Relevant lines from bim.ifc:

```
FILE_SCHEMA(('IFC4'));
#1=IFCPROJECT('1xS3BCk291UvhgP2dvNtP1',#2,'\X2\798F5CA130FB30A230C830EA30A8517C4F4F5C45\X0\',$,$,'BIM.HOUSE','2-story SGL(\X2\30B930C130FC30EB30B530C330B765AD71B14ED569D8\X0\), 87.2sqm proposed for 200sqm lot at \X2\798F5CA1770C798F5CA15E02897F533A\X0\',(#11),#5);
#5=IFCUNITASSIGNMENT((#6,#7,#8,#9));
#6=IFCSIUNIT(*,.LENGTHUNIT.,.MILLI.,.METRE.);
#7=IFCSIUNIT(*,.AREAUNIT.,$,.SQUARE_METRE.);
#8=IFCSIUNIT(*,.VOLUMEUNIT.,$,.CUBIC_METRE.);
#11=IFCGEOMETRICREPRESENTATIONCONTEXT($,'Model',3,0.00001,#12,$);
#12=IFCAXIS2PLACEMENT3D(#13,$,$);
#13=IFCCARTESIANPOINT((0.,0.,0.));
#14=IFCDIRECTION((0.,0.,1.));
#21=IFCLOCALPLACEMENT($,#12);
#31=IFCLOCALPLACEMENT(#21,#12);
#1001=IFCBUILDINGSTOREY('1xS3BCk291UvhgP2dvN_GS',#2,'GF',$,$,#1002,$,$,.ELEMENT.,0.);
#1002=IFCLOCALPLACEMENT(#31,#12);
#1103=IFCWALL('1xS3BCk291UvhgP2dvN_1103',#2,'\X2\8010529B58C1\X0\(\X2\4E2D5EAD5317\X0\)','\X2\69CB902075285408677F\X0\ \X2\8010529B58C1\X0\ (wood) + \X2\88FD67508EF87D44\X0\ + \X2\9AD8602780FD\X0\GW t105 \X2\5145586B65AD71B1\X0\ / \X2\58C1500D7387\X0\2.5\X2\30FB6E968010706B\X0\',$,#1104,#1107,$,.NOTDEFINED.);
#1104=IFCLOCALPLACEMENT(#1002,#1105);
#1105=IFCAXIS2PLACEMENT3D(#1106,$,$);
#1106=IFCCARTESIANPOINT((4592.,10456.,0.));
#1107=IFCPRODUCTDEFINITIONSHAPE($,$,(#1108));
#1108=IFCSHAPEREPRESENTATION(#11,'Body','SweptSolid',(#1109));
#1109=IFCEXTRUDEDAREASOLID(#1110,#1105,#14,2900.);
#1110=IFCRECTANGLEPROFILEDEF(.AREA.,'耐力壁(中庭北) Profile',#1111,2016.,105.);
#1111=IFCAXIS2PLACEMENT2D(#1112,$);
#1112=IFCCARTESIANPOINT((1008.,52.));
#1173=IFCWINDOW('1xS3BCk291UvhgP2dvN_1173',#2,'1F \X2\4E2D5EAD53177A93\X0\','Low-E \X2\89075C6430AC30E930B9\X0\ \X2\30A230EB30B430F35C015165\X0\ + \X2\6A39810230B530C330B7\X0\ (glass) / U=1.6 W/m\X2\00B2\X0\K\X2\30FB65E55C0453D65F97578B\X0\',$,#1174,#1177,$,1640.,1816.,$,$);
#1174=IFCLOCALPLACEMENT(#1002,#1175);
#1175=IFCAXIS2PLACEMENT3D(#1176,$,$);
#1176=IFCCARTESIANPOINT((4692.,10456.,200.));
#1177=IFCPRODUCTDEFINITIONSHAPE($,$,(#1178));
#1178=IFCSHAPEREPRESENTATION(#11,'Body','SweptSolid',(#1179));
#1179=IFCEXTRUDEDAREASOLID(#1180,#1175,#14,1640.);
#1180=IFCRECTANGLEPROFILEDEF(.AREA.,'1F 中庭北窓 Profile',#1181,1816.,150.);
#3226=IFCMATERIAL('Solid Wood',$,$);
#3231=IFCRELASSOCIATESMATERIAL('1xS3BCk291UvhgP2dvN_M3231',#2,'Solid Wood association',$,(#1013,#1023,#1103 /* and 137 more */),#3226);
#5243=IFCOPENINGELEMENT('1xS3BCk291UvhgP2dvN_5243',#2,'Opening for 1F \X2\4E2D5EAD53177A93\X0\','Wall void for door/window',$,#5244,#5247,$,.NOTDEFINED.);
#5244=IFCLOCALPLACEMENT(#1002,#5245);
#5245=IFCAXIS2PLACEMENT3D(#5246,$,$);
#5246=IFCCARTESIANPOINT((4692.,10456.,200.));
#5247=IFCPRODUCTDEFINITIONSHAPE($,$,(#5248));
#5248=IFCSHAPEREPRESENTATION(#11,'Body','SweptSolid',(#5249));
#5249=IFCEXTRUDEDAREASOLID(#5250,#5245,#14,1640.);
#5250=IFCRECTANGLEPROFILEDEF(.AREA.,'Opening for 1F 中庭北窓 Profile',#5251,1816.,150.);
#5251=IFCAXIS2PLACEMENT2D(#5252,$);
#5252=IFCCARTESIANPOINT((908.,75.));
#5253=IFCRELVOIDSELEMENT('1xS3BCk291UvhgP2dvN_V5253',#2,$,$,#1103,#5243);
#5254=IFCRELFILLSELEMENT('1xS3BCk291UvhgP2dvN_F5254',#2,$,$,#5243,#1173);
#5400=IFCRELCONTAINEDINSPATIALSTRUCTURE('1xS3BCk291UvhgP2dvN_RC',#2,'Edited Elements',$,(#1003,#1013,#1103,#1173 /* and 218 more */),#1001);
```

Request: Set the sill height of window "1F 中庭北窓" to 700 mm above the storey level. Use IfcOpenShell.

```python
import numpy as np
import ifcopenshell
import ifcopenshell.api.geometry
import ifcopenshell.geom
import ifcopenshell.util.element
import ifcopenshell.util.placement
import ifcopenshell.util.shape
import ifcopenshell.util.unit

model = ifcopenshell.open("bim.ifc")
unit_scale = ifcopenshell.util.unit.calculate_unit_scale(model)

window = model.by_guid("1xS3BCk291UvhgP2dvN_1173")
opening = window.FillsVoids[0].RelatingOpeningElement
storey = ifcopenshell.util.element.get_container(window, ifc_class="IfcBuildingStorey")
level = ifcopenshell.util.placement.get_local_placement(storey.ObjectPlacement)[2, 3]

# The opening's origin need not be at the sill, so measure its lowest point.
shape = ifcopenshell.geom.create_shape(ifcopenshell.geom.settings(), opening)
bottom = ifcopenshell.util.shape.get_shape_bottom_elevation(shape, shape.geometry) / unit_scale
dz = level + 0.7 / unit_scale - bottom

shift = np.array([0.0, 0.0, dz])
# The window is not placed relative to its opening, so move both.
for product in (opening, window):
    matrix = ifcopenshell.util.placement.get_local_placement(product.ObjectPlacement)
    matrix[:3, 3] += shift
    ifcopenshell.api.geometry.edit_object_placement(model, product=product, matrix=matrix, is_si=False)

print(f"moved by {dz * unit_scale:+.3f} m")

model.write("bim_edited.ifc")
```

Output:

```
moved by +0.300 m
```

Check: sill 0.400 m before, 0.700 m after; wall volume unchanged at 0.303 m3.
